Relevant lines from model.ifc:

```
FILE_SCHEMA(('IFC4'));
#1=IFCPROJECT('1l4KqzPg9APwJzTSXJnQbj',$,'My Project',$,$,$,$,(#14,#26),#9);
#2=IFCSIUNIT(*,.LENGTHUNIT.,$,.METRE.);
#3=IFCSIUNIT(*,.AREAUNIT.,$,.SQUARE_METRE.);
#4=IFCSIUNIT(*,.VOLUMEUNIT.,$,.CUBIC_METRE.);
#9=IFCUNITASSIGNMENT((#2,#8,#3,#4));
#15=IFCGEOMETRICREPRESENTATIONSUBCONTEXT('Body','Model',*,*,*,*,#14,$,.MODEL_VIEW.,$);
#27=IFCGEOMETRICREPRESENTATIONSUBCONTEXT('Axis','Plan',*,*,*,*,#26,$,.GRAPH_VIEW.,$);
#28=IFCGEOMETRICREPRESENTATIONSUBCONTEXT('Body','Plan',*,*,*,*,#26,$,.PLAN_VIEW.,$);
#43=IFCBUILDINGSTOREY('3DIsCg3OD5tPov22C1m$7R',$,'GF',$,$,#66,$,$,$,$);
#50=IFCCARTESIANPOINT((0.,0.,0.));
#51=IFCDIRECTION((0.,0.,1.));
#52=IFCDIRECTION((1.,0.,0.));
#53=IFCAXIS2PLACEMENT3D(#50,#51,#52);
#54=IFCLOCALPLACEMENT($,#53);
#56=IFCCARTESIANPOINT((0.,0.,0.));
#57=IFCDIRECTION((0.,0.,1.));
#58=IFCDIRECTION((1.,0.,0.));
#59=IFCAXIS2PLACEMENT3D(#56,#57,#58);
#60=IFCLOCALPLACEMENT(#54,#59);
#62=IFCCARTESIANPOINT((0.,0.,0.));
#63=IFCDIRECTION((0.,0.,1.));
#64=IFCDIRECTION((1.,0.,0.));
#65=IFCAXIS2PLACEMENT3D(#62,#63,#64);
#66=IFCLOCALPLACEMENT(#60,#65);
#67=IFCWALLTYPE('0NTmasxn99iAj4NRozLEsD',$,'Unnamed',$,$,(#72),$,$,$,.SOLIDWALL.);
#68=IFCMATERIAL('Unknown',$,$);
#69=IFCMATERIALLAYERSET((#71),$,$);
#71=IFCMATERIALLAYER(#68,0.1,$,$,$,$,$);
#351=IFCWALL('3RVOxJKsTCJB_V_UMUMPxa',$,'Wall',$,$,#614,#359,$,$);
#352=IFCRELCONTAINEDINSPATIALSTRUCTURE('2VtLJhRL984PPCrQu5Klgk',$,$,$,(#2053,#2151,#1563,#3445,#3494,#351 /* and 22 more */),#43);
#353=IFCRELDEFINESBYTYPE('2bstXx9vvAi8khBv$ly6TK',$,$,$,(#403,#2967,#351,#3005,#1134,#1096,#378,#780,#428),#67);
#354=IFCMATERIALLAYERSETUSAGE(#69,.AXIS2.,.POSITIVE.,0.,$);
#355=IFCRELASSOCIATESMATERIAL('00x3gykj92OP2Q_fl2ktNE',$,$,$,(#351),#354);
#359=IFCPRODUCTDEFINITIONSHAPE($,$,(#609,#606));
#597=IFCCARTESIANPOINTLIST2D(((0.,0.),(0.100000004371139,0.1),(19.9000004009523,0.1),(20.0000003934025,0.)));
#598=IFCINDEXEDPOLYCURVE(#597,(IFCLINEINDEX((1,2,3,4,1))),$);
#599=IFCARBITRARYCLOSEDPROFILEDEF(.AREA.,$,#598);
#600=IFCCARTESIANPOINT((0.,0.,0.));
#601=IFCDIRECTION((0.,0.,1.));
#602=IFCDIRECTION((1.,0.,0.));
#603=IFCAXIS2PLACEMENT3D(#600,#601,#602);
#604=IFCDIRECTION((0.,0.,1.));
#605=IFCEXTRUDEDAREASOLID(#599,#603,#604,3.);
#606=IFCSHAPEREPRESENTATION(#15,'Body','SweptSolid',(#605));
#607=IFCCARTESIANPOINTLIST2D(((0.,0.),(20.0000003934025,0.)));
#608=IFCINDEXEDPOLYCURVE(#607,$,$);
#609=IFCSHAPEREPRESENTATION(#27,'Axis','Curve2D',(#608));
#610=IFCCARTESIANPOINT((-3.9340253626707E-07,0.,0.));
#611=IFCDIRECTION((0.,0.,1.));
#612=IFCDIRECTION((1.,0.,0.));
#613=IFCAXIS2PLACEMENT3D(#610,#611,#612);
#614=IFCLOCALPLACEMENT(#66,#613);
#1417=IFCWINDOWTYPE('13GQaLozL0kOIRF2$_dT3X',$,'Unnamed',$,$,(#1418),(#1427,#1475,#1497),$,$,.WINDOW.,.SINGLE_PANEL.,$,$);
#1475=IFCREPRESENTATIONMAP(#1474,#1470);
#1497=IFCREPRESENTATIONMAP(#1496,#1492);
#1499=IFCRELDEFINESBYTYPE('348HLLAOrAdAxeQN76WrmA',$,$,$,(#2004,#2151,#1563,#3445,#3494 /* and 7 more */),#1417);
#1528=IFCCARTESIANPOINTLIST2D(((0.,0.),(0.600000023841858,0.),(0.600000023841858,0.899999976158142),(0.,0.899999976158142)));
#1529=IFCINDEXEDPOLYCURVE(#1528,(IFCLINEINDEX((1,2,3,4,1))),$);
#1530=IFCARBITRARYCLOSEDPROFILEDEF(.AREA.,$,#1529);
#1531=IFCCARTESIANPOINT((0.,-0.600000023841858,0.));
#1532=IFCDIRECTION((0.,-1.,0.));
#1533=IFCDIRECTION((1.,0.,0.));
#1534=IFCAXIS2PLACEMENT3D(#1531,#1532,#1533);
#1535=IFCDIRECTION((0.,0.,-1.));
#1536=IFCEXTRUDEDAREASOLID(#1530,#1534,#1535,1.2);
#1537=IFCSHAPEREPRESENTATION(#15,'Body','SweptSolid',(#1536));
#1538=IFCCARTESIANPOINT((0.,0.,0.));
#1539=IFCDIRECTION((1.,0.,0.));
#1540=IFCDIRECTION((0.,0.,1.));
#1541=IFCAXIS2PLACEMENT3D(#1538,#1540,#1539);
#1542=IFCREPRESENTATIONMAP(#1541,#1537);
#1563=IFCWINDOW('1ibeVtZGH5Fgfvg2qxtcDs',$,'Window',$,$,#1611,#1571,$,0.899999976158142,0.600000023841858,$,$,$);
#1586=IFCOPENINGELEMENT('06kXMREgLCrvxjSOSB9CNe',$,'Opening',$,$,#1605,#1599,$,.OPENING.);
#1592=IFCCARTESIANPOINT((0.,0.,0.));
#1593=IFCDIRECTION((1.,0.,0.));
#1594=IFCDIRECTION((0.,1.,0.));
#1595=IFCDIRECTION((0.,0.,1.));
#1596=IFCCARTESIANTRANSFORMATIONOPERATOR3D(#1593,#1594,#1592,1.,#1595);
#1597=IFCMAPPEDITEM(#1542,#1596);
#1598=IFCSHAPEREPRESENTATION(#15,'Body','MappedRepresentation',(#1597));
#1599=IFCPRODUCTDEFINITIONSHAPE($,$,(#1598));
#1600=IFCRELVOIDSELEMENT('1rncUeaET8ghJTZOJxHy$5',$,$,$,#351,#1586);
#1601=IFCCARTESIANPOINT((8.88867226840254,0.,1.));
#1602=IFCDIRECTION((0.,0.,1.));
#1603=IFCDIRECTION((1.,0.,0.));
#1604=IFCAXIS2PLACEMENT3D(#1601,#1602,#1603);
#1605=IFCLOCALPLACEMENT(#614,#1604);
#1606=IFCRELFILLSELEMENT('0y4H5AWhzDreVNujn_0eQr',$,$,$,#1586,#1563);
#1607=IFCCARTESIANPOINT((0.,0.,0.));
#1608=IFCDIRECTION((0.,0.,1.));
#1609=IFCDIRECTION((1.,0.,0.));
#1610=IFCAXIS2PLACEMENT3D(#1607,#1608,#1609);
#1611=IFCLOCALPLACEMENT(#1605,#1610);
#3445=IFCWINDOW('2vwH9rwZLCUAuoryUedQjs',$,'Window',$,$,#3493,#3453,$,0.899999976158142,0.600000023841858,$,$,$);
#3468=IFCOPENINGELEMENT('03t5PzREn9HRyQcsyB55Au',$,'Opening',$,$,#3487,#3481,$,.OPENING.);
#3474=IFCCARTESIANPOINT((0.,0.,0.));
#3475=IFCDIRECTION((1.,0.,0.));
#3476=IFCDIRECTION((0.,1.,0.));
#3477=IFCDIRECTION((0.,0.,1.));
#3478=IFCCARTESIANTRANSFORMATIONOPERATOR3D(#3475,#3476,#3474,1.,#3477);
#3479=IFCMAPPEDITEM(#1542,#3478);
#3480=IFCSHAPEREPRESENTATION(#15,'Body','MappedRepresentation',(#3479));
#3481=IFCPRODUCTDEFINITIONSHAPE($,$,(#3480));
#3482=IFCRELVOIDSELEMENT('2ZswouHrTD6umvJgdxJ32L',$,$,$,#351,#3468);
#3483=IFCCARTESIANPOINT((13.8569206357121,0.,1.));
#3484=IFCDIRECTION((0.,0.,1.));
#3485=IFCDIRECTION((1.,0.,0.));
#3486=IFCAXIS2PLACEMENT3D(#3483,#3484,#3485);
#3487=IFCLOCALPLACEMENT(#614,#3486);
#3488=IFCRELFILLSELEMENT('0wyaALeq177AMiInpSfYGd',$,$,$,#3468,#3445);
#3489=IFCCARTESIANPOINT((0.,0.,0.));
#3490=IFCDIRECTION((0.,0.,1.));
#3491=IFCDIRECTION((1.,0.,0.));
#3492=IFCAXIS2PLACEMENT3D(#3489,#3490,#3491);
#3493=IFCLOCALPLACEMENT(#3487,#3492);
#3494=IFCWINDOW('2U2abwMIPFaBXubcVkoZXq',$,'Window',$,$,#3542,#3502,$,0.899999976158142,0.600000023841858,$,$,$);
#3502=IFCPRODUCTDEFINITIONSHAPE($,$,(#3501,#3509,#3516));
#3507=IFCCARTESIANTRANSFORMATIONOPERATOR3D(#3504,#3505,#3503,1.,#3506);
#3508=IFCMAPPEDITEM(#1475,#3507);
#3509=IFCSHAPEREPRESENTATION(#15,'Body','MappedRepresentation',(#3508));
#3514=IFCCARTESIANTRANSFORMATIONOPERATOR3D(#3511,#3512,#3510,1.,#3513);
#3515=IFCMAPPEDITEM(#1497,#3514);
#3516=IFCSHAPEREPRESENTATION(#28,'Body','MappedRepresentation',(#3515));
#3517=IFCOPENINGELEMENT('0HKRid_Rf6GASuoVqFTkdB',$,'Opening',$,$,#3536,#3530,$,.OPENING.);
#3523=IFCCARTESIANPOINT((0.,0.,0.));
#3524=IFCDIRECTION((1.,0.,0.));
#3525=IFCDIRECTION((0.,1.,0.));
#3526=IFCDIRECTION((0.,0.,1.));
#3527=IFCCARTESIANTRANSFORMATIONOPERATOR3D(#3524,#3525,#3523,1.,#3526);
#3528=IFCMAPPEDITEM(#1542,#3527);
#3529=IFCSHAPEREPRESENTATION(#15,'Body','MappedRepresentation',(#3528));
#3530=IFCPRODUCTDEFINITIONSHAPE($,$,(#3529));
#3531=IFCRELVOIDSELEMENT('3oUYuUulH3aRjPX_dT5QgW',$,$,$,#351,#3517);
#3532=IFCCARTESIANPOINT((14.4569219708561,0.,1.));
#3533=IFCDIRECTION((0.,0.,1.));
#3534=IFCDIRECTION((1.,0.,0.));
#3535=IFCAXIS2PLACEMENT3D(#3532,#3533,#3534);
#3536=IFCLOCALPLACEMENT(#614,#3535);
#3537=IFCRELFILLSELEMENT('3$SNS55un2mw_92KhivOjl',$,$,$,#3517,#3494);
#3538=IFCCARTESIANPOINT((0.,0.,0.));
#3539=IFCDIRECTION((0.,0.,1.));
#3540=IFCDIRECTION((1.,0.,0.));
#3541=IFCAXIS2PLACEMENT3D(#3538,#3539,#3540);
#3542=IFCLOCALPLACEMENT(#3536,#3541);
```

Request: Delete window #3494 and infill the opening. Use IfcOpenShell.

```python
import ifcopenshell
import ifcopenshell.api.feature
import ifcopenshell.api.root
import ifcopenshell.geom
import ifcopenshell.util.shape

model = ifcopenshell.open("model.ifc")
settings = ifcopenshell.geom.settings()


def volume(element):
    """Net volume in cubic metres, openings subtracted."""
    shape = ifcopenshell.geom.create_shape(settings, element)
    return ifcopenshell.util.shape.get_volume(shape.geometry)


window = model.by_id(3494)
opening = window.FillsVoids[0].RelatingOpeningElement
wall = opening.VoidsElements[0].RelatingBuildingElement
before = volume(wall)

ifcopenshell.api.root.remove_product(model, product=window)
ifcopenshell.api.feature.remove_feature(model, feature=opening)

after = volume(wall)

print(f"wall volume {before:.3f} -> {after:.3f} m3")

model.write("model-out.ifc")
```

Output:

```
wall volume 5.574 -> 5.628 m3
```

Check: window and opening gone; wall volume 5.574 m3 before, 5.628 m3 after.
